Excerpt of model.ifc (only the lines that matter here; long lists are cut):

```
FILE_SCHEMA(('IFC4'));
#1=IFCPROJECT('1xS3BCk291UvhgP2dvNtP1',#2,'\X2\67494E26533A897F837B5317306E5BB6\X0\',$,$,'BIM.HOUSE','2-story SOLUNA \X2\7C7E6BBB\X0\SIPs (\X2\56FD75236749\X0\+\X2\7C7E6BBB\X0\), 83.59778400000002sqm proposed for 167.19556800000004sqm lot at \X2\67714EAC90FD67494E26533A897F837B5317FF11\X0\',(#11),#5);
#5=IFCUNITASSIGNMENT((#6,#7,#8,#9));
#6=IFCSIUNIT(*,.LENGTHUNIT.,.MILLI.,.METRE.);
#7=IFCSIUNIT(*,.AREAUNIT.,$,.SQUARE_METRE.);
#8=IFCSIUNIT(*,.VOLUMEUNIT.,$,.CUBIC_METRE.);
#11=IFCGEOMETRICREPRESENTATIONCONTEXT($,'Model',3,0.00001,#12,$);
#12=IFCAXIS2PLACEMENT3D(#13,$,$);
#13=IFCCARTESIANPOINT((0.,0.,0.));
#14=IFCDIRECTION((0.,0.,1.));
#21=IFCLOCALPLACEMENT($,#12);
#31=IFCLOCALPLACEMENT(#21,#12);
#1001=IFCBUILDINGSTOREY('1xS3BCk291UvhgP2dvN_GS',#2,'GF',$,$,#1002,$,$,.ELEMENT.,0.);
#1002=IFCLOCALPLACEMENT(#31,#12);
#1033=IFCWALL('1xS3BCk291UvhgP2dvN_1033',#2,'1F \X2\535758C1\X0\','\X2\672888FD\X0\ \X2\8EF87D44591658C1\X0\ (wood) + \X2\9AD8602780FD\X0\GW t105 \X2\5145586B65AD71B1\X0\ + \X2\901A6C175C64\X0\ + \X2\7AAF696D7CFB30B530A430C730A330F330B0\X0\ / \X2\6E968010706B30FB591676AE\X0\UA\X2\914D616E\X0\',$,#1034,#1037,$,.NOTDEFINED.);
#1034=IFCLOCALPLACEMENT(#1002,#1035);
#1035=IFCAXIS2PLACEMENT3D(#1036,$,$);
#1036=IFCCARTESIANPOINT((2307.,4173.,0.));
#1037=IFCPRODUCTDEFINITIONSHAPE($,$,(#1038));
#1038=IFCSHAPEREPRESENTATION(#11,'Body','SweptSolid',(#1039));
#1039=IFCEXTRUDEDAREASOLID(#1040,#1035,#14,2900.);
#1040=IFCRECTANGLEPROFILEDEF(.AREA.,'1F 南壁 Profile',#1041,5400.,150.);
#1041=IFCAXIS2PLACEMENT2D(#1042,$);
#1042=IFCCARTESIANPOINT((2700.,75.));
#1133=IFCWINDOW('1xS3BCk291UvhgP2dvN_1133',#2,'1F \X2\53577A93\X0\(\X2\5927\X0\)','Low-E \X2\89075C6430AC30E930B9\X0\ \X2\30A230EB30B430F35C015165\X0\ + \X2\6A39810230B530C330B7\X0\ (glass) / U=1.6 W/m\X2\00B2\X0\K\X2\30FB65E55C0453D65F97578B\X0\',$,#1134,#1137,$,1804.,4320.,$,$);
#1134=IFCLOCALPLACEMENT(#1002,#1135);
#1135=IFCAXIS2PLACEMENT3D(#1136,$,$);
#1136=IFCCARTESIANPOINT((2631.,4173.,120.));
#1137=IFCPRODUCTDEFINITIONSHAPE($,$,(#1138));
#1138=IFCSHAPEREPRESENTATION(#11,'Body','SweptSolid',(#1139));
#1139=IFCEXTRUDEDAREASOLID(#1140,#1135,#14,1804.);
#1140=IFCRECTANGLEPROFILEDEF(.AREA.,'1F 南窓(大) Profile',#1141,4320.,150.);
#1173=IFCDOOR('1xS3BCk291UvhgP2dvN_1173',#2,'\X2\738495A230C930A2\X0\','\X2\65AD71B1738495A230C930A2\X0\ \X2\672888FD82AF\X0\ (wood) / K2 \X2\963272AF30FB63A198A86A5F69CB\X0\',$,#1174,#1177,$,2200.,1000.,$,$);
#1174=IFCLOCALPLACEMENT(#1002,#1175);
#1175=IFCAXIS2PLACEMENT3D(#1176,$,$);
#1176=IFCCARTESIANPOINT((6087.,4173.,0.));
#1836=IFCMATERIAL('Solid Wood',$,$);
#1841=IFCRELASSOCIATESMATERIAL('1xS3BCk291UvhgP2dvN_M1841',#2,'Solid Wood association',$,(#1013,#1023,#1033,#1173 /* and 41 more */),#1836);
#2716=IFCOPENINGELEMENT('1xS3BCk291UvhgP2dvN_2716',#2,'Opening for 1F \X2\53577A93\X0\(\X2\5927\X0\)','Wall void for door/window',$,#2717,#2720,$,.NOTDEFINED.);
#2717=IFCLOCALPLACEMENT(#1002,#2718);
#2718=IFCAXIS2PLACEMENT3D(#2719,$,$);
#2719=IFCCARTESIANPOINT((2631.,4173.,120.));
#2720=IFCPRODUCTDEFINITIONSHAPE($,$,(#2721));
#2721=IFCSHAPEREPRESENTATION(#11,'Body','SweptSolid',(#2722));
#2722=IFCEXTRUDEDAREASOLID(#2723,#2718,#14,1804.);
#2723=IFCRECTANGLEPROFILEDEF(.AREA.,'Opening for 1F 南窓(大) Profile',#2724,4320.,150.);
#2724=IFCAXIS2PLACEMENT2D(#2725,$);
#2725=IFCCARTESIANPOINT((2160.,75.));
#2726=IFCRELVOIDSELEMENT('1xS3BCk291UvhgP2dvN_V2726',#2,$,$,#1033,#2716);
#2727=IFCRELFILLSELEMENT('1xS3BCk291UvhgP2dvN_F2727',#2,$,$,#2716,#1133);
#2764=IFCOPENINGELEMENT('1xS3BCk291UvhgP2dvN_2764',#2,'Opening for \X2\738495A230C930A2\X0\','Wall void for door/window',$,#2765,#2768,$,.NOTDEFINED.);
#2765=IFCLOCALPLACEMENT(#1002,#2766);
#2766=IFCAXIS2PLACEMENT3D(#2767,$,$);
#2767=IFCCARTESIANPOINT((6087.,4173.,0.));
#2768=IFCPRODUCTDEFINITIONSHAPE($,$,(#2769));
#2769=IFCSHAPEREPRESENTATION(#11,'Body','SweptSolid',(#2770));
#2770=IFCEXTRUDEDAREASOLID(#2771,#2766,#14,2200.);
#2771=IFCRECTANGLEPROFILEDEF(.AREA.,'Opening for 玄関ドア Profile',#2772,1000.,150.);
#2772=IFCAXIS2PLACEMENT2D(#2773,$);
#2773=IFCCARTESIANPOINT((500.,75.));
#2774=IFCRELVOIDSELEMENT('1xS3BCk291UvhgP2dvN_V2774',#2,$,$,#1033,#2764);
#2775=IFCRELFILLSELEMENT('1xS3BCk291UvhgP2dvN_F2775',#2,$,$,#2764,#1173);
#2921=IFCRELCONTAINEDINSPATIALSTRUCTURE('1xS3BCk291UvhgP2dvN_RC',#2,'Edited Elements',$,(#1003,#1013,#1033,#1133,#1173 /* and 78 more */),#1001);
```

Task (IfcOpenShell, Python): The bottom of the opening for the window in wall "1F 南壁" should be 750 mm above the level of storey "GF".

```python
import numpy as np
import ifcopenshell
import ifcopenshell.api.geometry
import ifcopenshell.geom
import ifcopenshell.util.element
import ifcopenshell.util.placement
import ifcopenshell.util.shape
import ifcopenshell.util.unit

model = ifcopenshell.open("model.ifc")
unit_scale = ifcopenshell.util.unit.calculate_unit_scale(model)

window = model.by_id(1133)
opening = window.FillsVoids[0].RelatingOpeningElement
storey = ifcopenshell.util.element.get_container(window, ifc_class="IfcBuildingStorey")
level = ifcopenshell.util.placement.get_local_placement(storey.ObjectPlacement)[2, 3]

# The opening's origin need not be at the sill, so measure its lowest point.
shape = ifcopenshell.geom.create_shape(ifcopenshell.geom.settings(), opening)
bottom = ifcopenshell.util.shape.get_shape_bottom_elevation(shape, shape.geometry) / unit_scale
dz = level + 0.75 / unit_scale - bottom

shift = np.array([0.0, 0.0, dz])
# The window is not placed relative to its opening, so move both.
for product in (opening, window):
    matrix = ifcopenshell.util.placement.get_local_placement(product.ObjectPlacement)
    matrix[:3, 3] += shift
    ifcopenshell.api.geometry.edit_object_placement(model, product=product, matrix=matrix, is_si=False)

print(f"moved by {dz * unit_scale:+.3f} m")

model.write("model_updated.ifc")
```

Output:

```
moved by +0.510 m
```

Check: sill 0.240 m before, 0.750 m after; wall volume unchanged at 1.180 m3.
